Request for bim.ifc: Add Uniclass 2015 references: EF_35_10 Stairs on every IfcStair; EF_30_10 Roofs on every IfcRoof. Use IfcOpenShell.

First a look at what the model holds.

```python
import ifcopenshell

model = ifcopenshell.open("bim.ifc")
print(model.schema)
print("classifications:", [c.Name for c in model.by_type("IfcClassification")])
for ifc_class in ("IfcDoor", "IfcRoof", "IfcStair", "IfcWall", "IfcWindow"):
    print(ifc_class, len(model.by_type(ifc_class)))
```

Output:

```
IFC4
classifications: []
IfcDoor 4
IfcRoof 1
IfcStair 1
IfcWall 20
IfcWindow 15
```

```python
import ifcopenshell
import ifcopenshell.api.classification

model = ifcopenshell.open("bim.ifc")

system = ifcopenshell.api.classification.add_classification(model, classification="Uniclass 2015")

codes = {
    "IfcStair": ("EF_35_10", "Stairs"),
    "IfcRoof": ("EF_30_10", "Roofs"),
}
for ifc_class, (code, name) in codes.items():
    products = model.by_type(ifc_class)
    ifcopenshell.api.classification.add_reference(
        model, products=products, classification=system, identification=code, name=name
    )
    print(code, len(products))

model.write("bim-out.ifc")
```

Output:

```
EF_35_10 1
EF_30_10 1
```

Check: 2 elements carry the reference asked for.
